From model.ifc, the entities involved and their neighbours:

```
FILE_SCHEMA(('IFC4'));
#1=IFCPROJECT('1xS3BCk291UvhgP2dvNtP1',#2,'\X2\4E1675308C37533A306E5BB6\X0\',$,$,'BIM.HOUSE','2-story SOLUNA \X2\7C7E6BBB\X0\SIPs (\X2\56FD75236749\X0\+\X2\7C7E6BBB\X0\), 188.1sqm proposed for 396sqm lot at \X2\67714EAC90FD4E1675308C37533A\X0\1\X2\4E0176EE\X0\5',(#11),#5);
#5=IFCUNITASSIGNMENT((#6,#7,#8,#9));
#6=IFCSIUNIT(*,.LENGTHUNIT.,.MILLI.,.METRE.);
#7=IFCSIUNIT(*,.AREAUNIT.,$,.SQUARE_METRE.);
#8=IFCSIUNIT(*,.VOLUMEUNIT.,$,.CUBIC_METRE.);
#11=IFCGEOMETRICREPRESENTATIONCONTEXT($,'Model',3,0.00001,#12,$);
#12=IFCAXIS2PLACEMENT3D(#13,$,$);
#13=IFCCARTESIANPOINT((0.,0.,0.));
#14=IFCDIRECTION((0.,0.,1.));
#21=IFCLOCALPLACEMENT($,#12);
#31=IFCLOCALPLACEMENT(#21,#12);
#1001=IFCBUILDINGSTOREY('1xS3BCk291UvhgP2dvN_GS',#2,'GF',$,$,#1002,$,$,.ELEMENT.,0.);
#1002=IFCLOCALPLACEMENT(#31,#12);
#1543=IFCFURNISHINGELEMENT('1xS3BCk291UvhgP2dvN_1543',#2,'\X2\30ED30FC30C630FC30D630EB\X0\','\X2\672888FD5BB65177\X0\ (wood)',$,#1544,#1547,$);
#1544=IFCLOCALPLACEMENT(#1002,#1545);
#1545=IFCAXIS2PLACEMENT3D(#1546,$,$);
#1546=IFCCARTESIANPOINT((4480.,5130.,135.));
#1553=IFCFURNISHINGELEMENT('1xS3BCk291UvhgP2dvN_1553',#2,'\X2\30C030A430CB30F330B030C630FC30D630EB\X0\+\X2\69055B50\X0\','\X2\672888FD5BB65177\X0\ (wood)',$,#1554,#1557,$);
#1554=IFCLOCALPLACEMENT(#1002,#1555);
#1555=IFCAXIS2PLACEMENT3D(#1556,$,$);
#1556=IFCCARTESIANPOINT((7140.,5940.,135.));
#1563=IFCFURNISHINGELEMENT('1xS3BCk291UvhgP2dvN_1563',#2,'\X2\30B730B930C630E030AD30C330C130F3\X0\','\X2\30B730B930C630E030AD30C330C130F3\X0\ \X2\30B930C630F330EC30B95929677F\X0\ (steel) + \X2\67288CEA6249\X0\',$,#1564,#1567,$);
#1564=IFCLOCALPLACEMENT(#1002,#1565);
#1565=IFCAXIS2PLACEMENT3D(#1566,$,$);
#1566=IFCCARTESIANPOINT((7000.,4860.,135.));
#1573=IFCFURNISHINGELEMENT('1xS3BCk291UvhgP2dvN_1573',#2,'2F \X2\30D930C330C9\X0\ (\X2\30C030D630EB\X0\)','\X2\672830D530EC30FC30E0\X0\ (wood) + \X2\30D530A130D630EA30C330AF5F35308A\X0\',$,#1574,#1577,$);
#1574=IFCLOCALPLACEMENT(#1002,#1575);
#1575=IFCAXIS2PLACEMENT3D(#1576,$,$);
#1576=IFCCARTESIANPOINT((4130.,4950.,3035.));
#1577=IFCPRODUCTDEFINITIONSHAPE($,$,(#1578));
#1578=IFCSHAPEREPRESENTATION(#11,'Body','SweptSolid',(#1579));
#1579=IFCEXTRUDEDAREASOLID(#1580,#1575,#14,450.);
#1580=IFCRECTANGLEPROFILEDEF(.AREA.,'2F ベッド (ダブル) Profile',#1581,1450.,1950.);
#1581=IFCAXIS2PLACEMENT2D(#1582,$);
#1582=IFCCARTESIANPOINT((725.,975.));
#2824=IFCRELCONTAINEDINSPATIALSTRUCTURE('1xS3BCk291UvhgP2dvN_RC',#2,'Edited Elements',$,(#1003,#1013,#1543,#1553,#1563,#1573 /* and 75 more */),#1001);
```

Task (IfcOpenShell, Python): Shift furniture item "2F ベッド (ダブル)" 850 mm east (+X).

```python
import ifcopenshell
import ifcopenshell.api.geometry
import ifcopenshell.util.placement
import ifcopenshell.util.unit

model = ifcopenshell.open("model.ifc")
unit_scale = ifcopenshell.util.unit.calculate_unit_scale(model)

item = model.by_id(1573)
matrix = ifcopenshell.util.placement.get_local_placement(item.ObjectPlacement)
matrix[0, 3] += 0.85 / unit_scale
ifcopenshell.api.geometry.edit_object_placement(model, product=item, matrix=matrix, is_si=False)

print(ifcopenshell.util.placement.get_local_placement(item.ObjectPlacement).round(3) + 0.0)

model.write("model_edited.ifc")
```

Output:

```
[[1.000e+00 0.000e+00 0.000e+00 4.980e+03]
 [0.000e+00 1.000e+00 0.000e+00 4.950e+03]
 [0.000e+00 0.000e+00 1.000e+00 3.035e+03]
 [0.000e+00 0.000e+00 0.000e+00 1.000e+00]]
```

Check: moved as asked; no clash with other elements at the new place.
